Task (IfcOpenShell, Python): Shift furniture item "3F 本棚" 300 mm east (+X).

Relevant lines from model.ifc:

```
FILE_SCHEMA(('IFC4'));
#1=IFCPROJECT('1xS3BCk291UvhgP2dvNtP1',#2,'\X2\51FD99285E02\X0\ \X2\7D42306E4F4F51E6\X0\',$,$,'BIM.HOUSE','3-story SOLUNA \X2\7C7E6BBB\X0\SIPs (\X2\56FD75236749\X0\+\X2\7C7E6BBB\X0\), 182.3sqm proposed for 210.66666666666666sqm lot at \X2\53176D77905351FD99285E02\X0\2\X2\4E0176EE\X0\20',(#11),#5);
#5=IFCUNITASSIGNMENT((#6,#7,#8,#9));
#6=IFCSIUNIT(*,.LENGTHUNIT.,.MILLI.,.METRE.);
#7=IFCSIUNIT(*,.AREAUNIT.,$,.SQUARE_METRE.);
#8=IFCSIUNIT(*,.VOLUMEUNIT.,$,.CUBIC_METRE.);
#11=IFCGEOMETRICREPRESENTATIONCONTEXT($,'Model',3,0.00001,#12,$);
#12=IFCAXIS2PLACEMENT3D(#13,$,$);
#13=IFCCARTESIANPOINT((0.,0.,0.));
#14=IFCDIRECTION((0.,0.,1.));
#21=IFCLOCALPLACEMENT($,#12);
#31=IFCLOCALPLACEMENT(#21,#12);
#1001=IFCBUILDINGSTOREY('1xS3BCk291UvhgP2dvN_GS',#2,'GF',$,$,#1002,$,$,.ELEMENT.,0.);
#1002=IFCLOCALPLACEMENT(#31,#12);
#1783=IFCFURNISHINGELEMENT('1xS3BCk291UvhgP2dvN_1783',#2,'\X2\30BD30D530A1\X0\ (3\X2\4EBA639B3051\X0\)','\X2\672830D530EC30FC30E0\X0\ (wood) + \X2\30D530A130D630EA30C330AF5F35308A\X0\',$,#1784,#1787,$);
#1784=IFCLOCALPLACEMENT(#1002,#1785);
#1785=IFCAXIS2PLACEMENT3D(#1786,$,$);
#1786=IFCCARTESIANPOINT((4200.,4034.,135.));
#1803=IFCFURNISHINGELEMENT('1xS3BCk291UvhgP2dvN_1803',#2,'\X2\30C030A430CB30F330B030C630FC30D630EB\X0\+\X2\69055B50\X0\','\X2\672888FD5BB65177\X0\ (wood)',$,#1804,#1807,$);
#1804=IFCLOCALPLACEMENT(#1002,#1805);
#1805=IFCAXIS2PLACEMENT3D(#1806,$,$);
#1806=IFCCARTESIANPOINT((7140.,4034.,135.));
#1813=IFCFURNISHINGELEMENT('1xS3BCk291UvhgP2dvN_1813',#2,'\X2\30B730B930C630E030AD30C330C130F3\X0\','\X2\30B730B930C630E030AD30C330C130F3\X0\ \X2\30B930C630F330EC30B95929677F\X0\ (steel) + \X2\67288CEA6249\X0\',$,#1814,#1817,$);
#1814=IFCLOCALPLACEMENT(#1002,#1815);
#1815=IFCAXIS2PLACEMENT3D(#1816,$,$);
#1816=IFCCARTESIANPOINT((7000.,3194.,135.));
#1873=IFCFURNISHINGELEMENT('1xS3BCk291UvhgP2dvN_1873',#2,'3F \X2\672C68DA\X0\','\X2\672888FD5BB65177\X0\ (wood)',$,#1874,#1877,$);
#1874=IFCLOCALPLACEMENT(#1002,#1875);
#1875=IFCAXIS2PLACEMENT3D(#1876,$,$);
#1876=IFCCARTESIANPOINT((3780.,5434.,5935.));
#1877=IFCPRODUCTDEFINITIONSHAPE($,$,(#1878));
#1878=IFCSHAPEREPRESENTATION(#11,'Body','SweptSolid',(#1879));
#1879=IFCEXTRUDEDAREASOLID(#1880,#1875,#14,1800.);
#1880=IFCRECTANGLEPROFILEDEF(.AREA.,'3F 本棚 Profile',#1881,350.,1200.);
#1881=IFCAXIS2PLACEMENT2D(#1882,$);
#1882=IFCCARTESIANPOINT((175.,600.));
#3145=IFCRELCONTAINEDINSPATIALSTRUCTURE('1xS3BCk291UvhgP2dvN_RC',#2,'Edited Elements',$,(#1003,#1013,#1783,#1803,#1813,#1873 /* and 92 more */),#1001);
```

```python
import ifcopenshell
import ifcopenshell.api.geometry
import ifcopenshell.util.placement
import ifcopenshell.util.unit

model = ifcopenshell.open("model.ifc")
unit_scale = ifcopenshell.util.unit.calculate_unit_scale(model)

item = model.by_id(1873)
matrix = ifcopenshell.util.placement.get_local_placement(item.ObjectPlacement)
matrix[0, 3] += 0.3 / unit_scale
ifcopenshell.api.geometry.edit_object_placement(model, product=item, matrix=matrix, is_si=False)

print(ifcopenshell.util.placement.get_local_placement(item.ObjectPlacement).round(3) + 0.0)

model.write("model_edited.ifc")
```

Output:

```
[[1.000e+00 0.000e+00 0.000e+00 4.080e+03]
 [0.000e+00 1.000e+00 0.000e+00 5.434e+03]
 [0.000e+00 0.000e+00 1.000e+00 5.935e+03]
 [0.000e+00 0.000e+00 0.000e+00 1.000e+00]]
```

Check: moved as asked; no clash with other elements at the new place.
